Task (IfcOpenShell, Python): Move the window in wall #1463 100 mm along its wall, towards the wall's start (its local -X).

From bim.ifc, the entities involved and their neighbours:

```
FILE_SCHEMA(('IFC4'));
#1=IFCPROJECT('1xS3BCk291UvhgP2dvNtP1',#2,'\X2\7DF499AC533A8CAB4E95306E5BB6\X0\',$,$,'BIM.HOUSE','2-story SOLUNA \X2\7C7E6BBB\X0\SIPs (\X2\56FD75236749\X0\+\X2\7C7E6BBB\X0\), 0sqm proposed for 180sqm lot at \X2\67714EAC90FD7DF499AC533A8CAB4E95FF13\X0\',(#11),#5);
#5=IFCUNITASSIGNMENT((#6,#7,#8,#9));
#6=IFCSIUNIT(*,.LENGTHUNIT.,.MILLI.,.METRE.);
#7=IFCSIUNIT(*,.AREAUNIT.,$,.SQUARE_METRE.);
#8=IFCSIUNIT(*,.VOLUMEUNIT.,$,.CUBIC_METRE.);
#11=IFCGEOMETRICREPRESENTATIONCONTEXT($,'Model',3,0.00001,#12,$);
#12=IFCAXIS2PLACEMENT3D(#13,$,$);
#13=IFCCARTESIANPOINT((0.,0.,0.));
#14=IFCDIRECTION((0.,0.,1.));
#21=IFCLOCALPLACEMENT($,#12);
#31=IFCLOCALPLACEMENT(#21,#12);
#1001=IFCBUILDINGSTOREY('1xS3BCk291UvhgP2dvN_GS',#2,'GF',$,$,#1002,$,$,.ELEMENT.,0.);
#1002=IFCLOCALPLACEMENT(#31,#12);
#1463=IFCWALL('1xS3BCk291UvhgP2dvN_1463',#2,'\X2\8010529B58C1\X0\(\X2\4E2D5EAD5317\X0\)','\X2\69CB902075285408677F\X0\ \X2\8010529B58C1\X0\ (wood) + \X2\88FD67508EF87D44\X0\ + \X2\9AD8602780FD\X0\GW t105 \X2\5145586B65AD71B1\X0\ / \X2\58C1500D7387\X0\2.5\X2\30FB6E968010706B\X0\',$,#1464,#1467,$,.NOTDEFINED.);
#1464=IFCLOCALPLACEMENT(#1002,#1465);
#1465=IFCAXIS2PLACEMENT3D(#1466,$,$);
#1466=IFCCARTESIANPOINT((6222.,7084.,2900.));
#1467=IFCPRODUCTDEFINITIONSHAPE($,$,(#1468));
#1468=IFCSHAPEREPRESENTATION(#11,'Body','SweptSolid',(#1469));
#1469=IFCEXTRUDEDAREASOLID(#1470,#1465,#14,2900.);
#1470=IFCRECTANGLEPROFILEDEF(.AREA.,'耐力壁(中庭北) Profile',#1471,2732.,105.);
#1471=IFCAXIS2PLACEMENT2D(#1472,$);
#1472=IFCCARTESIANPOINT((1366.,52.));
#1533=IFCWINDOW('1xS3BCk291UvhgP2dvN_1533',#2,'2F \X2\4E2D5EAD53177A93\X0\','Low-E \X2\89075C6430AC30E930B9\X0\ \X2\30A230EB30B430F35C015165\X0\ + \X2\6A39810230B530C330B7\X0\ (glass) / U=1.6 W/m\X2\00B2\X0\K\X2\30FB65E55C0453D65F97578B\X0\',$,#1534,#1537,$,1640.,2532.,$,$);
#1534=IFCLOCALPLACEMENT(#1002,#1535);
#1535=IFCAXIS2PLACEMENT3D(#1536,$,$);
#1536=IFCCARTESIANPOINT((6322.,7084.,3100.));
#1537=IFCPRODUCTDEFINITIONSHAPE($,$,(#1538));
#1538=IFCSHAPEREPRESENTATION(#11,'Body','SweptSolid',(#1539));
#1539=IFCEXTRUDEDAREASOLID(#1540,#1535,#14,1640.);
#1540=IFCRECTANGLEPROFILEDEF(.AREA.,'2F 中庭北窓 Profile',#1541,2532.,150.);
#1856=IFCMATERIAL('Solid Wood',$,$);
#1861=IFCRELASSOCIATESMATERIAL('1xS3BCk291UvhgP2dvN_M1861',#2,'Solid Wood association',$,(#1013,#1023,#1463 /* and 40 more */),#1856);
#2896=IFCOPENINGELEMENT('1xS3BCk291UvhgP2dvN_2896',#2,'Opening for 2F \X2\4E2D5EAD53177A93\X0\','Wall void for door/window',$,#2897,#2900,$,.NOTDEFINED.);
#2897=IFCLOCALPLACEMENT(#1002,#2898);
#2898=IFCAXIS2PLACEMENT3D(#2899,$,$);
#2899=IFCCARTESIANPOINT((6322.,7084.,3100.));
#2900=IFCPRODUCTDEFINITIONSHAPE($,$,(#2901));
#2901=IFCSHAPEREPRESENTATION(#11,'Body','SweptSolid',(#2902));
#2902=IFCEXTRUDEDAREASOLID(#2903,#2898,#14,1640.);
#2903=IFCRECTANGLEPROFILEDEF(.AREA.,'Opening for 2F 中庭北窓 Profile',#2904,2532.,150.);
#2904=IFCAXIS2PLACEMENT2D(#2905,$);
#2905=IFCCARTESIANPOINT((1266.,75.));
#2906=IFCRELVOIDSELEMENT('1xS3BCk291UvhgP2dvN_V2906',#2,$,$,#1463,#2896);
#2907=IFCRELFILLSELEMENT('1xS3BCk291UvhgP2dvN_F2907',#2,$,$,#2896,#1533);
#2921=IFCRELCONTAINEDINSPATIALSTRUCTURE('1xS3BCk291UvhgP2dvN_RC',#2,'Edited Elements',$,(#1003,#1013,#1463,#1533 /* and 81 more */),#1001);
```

```python
import ifcopenshell
import ifcopenshell.api.geometry
import ifcopenshell.util.placement

model = ifcopenshell.open("bim.ifc")

window = model.by_guid("1xS3BCk291UvhgP2dvN_1533")
opening = window.FillsVoids[0].RelatingOpeningElement
wall = opening.VoidsElements[0].RelatingBuildingElement

wall_matrix = ifcopenshell.util.placement.get_local_placement(wall.ObjectPlacement)
shift = wall_matrix[:3, 0] * -100.0
before = ifcopenshell.util.placement.get_local_placement(window.ObjectPlacement)[:3, 3].copy()

# The window is not placed relative to its opening, so move both.
for product in (opening, window):
    matrix = ifcopenshell.util.placement.get_local_placement(product.ObjectPlacement)
    matrix[:3, 3] += shift
    ifcopenshell.api.geometry.edit_object_placement(model, product=product, matrix=matrix, is_si=False)

after = ifcopenshell.util.placement.get_local_placement(window.ObjectPlacement)[:3, 3]
print("window moved by", (after - before).round(3) + 0.0)

model.write("bim-out.ifc")
```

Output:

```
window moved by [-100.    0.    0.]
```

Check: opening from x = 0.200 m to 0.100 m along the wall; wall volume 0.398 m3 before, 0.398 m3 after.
